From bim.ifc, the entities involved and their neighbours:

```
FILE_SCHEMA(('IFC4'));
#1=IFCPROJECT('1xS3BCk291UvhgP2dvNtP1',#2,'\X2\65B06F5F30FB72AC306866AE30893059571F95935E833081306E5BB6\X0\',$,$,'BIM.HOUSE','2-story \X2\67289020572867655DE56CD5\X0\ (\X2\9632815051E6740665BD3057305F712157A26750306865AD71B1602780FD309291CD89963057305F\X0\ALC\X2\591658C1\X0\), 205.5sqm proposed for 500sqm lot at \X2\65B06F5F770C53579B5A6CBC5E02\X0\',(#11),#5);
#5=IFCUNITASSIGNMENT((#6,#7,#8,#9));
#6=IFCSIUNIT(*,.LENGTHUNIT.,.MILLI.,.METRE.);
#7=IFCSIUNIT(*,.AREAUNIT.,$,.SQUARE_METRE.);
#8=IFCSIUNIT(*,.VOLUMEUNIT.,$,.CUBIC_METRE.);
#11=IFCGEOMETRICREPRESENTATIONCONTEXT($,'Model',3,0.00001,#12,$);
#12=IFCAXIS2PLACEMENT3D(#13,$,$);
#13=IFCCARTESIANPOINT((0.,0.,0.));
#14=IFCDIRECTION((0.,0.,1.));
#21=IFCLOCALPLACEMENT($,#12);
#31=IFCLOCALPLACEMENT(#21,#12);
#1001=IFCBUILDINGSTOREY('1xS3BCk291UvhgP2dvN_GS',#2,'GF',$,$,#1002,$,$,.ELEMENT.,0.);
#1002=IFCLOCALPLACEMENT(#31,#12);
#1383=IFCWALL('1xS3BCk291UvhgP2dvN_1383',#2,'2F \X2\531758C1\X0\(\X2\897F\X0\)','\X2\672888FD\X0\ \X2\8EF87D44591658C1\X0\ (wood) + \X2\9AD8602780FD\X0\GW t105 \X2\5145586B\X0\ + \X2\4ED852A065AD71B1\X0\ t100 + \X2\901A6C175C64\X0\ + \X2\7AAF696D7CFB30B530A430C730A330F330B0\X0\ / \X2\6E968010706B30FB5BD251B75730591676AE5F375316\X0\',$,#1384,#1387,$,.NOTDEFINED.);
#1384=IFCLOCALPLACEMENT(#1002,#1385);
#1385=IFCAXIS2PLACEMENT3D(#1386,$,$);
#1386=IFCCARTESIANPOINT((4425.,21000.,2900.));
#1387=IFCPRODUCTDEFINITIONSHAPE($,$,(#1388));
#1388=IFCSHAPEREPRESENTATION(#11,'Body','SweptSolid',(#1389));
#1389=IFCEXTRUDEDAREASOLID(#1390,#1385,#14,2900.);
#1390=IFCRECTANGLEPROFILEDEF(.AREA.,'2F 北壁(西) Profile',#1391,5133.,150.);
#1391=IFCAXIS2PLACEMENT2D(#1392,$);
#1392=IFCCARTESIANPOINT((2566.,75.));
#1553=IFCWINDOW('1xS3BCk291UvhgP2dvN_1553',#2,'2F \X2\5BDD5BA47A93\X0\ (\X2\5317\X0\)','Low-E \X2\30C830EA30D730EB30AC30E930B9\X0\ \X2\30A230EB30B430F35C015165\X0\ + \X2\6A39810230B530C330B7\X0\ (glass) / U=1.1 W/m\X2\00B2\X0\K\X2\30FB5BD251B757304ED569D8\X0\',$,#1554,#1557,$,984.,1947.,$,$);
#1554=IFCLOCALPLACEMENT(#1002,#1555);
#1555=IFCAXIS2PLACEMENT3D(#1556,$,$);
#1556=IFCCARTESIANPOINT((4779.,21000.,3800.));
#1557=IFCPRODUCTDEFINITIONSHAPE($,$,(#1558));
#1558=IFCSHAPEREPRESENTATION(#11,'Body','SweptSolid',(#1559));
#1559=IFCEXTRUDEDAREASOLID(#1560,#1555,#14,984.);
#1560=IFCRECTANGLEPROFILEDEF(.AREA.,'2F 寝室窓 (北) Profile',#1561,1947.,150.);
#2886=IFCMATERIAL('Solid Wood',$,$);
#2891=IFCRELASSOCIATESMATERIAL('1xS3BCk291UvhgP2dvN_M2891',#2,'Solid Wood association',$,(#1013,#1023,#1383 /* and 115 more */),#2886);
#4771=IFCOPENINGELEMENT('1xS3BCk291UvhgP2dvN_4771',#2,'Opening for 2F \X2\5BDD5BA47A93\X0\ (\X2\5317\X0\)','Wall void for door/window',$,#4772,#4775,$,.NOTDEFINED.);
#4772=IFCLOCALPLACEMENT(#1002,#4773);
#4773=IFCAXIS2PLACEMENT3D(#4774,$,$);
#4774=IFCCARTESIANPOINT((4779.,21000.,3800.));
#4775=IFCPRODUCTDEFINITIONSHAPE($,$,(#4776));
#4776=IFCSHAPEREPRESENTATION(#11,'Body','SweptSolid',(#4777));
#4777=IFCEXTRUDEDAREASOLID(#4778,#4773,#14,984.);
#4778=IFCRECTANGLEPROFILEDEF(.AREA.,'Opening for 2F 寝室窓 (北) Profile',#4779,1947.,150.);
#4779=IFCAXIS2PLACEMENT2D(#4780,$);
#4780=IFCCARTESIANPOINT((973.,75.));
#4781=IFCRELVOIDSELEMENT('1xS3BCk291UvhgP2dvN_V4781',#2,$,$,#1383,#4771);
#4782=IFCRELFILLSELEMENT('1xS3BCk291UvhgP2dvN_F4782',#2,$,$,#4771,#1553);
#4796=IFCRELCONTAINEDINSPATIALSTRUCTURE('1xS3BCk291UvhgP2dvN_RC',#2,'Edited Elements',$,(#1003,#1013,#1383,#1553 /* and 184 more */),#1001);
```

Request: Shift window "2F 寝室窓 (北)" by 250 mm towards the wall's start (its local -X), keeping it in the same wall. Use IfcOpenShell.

```python
import ifcopenshell
import ifcopenshell.api.geometry
import ifcopenshell.util.placement
import ifcopenshell.util.unit

model = ifcopenshell.open("bim.ifc")
unit_scale = ifcopenshell.util.unit.calculate_unit_scale(model)

window = model.by_guid("1xS3BCk291UvhgP2dvN_1553")
opening = window.FillsVoids[0].RelatingOpeningElement
wall = opening.VoidsElements[0].RelatingBuildingElement

wall_matrix = ifcopenshell.util.placement.get_local_placement(wall.ObjectPlacement)
shift = wall_matrix[:3, 0] * -0.25 / unit_scale
before = ifcopenshell.util.placement.get_local_placement(window.ObjectPlacement)[:3, 3].copy()

# The window is not placed relative to its opening, so move both.
for product in (opening, window):
    matrix = ifcopenshell.util.placement.get_local_placement(product.ObjectPlacement)
    matrix[:3, 3] += shift
    ifcopenshell.api.geometry.edit_object_placement(model, product=product, matrix=matrix, is_si=False)

after = ifcopenshell.util.placement.get_local_placement(window.ObjectPlacement)[:3, 3]
print("window moved by", (after - before).round(3) + 0.0)

model.write("bim_rev.ifc")
```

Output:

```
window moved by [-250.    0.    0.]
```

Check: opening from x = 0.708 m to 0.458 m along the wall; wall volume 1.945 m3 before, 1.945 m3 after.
